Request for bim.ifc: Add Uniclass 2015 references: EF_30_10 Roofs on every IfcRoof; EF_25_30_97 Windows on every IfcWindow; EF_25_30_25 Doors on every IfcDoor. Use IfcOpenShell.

First a look at what the model holds.

```python
import ifcopenshell

model = ifcopenshell.open("bim.ifc")
print(model.schema)
print("classifications:", [c.Name for c in model.by_type("IfcClassification")])
for ifc_class in ("IfcDoor", "IfcRoof", "IfcStair", "IfcWall", "IfcWindow"):
    print(ifc_class, len(model.by_type(ifc_class)))
```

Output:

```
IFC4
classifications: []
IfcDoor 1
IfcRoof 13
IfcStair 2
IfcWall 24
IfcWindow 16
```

```python
import ifcopenshell
import ifcopenshell.api.classification

model = ifcopenshell.open("bim.ifc")

system = ifcopenshell.api.classification.add_classification(model, classification="Uniclass 2015")

codes = {
    "IfcRoof": ("EF_30_10", "Roofs"),
    "IfcWindow": ("EF_25_30_97", "Windows"),
    "IfcDoor": ("EF_25_30_25", "Doors"),
}
for ifc_class, (code, name) in codes.items():
    products = model.by_type(ifc_class)
    ifcopenshell.api.classification.add_reference(
        model, products=products, classification=system, identification=code, name=name
    )
    print(code, len(products))

model.write("bim_edited.ifc")
```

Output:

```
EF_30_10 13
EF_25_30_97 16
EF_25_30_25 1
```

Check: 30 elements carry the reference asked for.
